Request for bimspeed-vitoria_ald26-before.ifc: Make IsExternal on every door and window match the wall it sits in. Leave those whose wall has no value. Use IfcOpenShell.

First a look at what the model holds.

```python
import ifcopenshell
import ifcopenshell.util.element

model = ifcopenshell.open("bimspeed-vitoria_ald26-before.ifc")
print(model.schema)
seen = {}
for e in model.by_type("IfcDoor") + model.by_type("IfcWindow"):
    if not e.FillsVoids:
        continue
    host = e.FillsVoids[0].RelatingOpeningElement.VoidsElements[0].RelatingBuildingElement
    own = ifcopenshell.util.element.get_pset(e, f"Pset_{e.is_a()[3:].removesuffix('StandardCase')}Common", "IsExternal")
    wall = ifcopenshell.util.element.get_pset(host, "Pset_WallCommon", "IsExternal")
    seen[e.is_a(), own, wall] = seen.get((e.is_a(), own, wall), 0) + 1
for (cls, own, wall), count in sorted(seen.items(), key=str):
    print(count, cls, "IsExternal:", own, "| host wall:", wall)
```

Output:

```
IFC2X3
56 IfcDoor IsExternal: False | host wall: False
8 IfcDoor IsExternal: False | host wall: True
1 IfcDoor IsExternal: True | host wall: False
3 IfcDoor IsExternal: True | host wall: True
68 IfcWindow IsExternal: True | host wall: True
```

```python
import ifcopenshell
import ifcopenshell.api.pset
import ifcopenshell.util.element

model = ifcopenshell.open("bimspeed-vitoria_ald26-before.ifc")

count = 0
for ifc_class, pset_name in (("IfcDoor", "Pset_DoorCommon"), ("IfcWindow", "Pset_WindowCommon")):
    for e in model.by_type(ifc_class):
        if not e.FillsVoids:
            continue
        host = e.FillsVoids[0].RelatingOpeningElement.VoidsElements[0].RelatingBuildingElement
        external = ifcopenshell.util.element.get_pset(host, "Pset_WallCommon", "IsExternal")
        if external is None or ifcopenshell.util.element.get_pset(e, pset_name, "IsExternal") == external:
            continue
        pset = ifcopenshell.api.pset.add_pset(model, product=e, name=pset_name)
        ifcopenshell.api.pset.edit_pset(model, pset=pset, properties={"IsExternal": external})
        count += 1

print(count, "updated")

model.write("bimspeed-vitoria_ald26-before_updated.ifc")
```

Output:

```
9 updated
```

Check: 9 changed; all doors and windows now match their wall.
